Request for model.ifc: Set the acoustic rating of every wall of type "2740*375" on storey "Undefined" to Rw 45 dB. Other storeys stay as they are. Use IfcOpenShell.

First a look at what the model holds.

```python
import ifcopenshell
import ifcopenshell.util.element

model = ifcopenshell.open("model.ifc")
print(model.schema)
storey = next(s for s in model.by_type("IfcBuildingStorey") if s.Name == "Undefined")
walls = [e for e in ifcopenshell.util.element.get_decomposition(storey) if e.is_a("IfcWall")]
seen = {}
for e in walls:
    element_type = ifcopenshell.util.element.get_type(e)
    key = (element_type.Name if element_type != e and element_type else None, ifcopenshell.util.element.get_pset(e, "Pset_WallCommon", "AcousticRating"))
    seen[key] = seen.get(key, 0) + 1
for (name, value), count in sorted(seen.items(), key=str):
    print(count, "x", name, "|", value)
```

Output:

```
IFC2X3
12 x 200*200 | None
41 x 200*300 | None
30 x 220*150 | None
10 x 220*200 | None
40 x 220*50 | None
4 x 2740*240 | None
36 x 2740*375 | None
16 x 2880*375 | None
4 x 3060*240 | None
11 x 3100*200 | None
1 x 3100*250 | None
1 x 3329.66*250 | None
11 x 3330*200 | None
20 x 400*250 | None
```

```python
import ifcopenshell
import ifcopenshell.api.pset
import ifcopenshell.util.element

model = ifcopenshell.open("model.ifc")

storey = next(s for s in model.by_type("IfcBuildingStorey") if s.Name == "Undefined")
walls = [e for e in ifcopenshell.util.element.get_decomposition(storey) if e.is_a("IfcWall")]

count = 0
for e in walls:
    element_type = ifcopenshell.util.element.get_type(e)
    if element_type in (None, e) or element_type.Name != "2740*375":
        continue
    # add_pset returns the element's existing set when there is one.
    pset = ifcopenshell.api.pset.add_pset(model, product=e, name="Pset_WallCommon")
    ifcopenshell.api.pset.edit_pset(model, pset=pset, properties={"AcousticRating": "Rw 45 dB"})
    count += 1

print(count, "walls updated")

model.write("model-out.ifc")
```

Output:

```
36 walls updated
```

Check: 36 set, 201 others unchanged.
